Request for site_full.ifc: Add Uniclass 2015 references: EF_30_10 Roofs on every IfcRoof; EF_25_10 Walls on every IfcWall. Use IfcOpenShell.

First a look at what the model holds.

```python
import ifcopenshell

model = ifcopenshell.open("site_full.ifc")
print(model.schema)
print("classifications:", [c.Name for c in model.by_type("IfcClassification")])
for ifc_class in ("IfcDoor", "IfcRoof", "IfcStair", "IfcWall", "IfcWindow"):
    print(ifc_class, len(model.by_type(ifc_class)))
```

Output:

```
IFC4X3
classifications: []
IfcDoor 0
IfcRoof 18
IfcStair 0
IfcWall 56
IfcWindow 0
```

```python
import ifcopenshell
import ifcopenshell.api.classification

model = ifcopenshell.open("site_full.ifc")

system = ifcopenshell.api.classification.add_classification(model, classification="Uniclass 2015")

codes = {
    "IfcRoof": ("EF_30_10", "Roofs"),
    "IfcWall": ("EF_25_10", "Walls"),
}
for ifc_class, (code, name) in codes.items():
    products = model.by_type(ifc_class)
    ifcopenshell.api.classification.add_reference(
        model, products=products, classification=system, identification=code, name=name
    )
    print(code, len(products))

model.write("site_full_updated.ifc")
```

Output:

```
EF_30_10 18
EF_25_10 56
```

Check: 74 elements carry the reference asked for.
